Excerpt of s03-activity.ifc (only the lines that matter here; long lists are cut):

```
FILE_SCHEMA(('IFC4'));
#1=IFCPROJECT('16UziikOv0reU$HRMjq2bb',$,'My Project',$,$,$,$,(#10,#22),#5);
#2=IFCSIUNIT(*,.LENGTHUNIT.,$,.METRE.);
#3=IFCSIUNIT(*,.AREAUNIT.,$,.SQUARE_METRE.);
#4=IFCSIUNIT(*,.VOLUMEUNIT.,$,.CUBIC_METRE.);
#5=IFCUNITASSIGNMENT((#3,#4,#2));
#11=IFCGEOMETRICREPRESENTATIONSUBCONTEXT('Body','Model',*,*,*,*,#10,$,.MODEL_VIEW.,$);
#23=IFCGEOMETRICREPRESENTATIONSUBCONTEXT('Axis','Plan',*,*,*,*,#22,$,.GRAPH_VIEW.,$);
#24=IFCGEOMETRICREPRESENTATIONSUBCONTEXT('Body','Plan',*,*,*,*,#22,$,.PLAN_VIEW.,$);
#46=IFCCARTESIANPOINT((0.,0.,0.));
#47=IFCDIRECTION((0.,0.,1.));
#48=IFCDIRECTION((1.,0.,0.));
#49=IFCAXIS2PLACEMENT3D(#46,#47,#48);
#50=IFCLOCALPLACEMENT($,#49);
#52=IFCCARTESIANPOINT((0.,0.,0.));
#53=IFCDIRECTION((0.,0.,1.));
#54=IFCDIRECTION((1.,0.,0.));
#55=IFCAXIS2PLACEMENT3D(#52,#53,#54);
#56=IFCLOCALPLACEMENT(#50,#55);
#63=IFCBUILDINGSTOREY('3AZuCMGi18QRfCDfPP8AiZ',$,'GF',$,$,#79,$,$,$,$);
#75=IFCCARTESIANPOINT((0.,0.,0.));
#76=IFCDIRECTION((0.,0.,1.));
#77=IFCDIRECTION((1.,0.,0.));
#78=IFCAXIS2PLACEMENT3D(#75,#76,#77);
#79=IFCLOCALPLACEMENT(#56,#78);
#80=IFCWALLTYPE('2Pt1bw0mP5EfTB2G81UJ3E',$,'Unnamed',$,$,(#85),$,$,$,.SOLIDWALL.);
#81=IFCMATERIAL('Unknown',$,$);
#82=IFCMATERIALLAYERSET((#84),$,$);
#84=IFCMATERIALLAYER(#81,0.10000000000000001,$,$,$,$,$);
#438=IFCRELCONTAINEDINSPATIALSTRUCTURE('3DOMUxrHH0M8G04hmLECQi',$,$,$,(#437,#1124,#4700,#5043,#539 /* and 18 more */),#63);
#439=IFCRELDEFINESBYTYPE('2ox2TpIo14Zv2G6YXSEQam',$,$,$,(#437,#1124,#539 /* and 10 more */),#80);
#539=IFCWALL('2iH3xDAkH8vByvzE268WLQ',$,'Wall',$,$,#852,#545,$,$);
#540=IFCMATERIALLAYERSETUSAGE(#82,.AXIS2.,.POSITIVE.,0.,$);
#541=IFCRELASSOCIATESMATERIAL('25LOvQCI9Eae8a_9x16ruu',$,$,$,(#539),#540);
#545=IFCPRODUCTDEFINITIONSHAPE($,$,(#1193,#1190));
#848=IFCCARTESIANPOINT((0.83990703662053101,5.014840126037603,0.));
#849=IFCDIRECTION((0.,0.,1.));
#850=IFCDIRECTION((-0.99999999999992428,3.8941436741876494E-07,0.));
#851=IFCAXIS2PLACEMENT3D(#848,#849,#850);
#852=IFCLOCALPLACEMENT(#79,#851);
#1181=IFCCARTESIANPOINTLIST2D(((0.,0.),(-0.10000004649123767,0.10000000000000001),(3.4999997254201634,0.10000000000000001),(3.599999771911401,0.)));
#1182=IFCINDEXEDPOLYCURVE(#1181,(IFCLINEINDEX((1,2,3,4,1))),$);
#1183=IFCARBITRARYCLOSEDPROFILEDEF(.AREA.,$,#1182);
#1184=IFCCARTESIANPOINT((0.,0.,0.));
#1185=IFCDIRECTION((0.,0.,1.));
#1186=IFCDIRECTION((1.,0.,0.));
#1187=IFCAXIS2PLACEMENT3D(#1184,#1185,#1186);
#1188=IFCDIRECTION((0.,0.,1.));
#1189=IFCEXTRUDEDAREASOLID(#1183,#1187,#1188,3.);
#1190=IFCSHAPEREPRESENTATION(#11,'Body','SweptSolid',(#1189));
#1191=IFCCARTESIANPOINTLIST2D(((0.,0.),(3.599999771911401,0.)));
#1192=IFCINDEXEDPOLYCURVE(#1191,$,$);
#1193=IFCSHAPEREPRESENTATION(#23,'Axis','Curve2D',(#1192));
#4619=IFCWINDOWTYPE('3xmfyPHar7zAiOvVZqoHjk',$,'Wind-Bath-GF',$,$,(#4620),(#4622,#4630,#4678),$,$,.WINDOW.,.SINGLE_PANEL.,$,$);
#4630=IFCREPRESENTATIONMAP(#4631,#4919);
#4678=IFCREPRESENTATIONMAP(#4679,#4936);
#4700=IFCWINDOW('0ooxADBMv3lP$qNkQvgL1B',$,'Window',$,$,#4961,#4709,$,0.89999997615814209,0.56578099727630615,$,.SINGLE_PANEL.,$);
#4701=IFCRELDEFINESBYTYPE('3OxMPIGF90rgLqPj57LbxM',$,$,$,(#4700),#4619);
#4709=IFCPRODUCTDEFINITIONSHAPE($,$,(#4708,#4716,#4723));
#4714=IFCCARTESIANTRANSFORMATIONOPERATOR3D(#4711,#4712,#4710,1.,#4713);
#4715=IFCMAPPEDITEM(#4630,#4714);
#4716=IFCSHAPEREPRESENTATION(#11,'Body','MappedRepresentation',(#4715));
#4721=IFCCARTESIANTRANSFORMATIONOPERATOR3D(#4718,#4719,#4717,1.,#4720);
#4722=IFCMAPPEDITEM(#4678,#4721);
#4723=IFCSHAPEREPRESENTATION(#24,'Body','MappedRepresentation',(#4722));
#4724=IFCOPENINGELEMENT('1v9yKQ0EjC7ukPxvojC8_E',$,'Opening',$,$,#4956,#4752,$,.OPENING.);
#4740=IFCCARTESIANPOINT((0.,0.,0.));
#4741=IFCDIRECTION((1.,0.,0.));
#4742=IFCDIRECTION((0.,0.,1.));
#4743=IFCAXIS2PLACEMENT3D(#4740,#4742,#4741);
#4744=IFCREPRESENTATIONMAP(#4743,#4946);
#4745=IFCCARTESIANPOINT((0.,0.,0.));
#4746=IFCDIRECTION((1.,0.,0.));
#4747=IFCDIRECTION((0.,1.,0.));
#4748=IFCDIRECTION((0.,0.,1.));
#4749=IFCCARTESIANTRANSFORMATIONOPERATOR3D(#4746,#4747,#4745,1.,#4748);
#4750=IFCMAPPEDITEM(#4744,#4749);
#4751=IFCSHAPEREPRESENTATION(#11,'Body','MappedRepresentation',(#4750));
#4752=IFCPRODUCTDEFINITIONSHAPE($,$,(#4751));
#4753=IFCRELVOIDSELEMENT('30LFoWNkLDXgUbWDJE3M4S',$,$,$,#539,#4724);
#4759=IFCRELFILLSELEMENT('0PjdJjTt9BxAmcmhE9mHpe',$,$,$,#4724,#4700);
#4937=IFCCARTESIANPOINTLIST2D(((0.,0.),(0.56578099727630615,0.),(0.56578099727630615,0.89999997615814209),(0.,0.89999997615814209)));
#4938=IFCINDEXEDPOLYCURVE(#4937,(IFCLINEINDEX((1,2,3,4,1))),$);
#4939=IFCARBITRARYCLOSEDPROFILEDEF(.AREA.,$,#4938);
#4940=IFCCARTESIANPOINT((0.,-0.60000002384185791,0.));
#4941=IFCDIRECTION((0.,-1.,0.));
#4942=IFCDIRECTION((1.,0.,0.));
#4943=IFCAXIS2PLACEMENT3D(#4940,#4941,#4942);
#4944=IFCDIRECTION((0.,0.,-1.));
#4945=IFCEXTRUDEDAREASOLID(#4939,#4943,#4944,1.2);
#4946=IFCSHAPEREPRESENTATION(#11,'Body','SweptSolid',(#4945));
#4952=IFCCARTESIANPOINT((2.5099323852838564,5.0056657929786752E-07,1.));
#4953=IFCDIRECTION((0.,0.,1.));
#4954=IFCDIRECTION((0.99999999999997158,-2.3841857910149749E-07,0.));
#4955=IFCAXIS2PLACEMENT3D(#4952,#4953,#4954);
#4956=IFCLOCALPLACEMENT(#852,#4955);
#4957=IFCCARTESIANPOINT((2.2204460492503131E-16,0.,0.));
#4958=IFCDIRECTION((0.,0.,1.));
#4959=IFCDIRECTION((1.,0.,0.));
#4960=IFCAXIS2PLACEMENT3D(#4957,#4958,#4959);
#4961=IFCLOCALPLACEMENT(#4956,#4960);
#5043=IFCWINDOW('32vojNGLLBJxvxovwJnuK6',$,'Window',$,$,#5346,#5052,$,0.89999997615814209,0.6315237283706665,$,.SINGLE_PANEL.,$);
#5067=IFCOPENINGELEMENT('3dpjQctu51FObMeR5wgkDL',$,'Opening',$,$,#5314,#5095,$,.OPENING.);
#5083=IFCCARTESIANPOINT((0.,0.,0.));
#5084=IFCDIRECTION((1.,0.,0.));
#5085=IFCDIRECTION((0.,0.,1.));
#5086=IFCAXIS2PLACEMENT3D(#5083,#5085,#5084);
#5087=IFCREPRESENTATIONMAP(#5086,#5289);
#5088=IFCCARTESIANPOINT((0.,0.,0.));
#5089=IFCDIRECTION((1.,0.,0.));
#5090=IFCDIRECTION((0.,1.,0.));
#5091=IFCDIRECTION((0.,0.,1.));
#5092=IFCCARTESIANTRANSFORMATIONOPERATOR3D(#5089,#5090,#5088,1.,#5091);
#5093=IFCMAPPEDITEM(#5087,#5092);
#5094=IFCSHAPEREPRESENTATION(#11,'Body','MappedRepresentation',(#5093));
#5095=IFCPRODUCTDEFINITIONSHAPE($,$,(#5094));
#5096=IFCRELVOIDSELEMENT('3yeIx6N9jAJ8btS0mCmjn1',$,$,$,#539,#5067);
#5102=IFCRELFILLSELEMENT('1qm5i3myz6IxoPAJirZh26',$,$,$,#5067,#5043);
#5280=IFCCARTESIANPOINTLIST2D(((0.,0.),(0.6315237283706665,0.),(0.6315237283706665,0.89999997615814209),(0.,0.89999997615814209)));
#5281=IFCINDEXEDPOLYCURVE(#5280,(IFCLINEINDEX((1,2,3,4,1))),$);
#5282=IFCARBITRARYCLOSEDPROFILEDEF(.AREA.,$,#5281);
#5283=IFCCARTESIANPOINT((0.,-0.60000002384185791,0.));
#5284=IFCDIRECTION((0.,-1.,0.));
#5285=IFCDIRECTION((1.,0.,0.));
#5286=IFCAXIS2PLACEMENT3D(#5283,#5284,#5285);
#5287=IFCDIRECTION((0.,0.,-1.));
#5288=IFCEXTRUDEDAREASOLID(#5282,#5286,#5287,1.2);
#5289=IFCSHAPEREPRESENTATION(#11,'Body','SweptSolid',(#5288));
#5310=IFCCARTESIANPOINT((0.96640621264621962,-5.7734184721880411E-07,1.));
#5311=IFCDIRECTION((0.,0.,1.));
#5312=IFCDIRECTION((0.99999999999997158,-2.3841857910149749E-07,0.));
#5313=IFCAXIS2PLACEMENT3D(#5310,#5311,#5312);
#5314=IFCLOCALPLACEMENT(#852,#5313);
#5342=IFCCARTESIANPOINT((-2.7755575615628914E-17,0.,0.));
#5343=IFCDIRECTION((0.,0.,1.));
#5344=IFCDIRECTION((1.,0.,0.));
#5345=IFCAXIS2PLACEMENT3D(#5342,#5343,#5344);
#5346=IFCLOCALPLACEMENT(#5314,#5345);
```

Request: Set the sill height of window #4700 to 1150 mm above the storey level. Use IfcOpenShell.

```python
import numpy as np
import ifcopenshell
import ifcopenshell.api.geometry
import ifcopenshell.geom
import ifcopenshell.util.element
import ifcopenshell.util.placement
import ifcopenshell.util.shape
import ifcopenshell.util.unit

model = ifcopenshell.open("s03-activity.ifc")
unit_scale = ifcopenshell.util.unit.calculate_unit_scale(model)

window = model.by_guid("0ooxADBMv3lP$qNkQvgL1B")
opening = window.FillsVoids[0].RelatingOpeningElement
storey = ifcopenshell.util.element.get_container(window, ifc_class="IfcBuildingStorey")
level = ifcopenshell.util.placement.get_local_placement(storey.ObjectPlacement)[2, 3]

# The opening's origin need not be at the sill, so measure its lowest point.
shape = ifcopenshell.geom.create_shape(ifcopenshell.geom.settings(), opening)
bottom = ifcopenshell.util.shape.get_shape_bottom_elevation(shape, shape.geometry) / unit_scale
dz = level + 1.15 - bottom

shift = np.array([0.0, 0.0, dz])
# The window is placed relative to its opening, so it follows when the opening moves.
matrix = ifcopenshell.util.placement.get_local_placement(opening.ObjectPlacement)
matrix[:3, 3] += shift
ifcopenshell.api.geometry.edit_object_placement(
    model, product=opening, matrix=matrix, is_si=False, should_transform_children=True
)

print(f"moved by {dz * unit_scale:+.3f} m")

model.write("s03-activity-out.ifc")
```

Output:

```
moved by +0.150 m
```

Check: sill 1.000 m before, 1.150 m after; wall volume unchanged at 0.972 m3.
